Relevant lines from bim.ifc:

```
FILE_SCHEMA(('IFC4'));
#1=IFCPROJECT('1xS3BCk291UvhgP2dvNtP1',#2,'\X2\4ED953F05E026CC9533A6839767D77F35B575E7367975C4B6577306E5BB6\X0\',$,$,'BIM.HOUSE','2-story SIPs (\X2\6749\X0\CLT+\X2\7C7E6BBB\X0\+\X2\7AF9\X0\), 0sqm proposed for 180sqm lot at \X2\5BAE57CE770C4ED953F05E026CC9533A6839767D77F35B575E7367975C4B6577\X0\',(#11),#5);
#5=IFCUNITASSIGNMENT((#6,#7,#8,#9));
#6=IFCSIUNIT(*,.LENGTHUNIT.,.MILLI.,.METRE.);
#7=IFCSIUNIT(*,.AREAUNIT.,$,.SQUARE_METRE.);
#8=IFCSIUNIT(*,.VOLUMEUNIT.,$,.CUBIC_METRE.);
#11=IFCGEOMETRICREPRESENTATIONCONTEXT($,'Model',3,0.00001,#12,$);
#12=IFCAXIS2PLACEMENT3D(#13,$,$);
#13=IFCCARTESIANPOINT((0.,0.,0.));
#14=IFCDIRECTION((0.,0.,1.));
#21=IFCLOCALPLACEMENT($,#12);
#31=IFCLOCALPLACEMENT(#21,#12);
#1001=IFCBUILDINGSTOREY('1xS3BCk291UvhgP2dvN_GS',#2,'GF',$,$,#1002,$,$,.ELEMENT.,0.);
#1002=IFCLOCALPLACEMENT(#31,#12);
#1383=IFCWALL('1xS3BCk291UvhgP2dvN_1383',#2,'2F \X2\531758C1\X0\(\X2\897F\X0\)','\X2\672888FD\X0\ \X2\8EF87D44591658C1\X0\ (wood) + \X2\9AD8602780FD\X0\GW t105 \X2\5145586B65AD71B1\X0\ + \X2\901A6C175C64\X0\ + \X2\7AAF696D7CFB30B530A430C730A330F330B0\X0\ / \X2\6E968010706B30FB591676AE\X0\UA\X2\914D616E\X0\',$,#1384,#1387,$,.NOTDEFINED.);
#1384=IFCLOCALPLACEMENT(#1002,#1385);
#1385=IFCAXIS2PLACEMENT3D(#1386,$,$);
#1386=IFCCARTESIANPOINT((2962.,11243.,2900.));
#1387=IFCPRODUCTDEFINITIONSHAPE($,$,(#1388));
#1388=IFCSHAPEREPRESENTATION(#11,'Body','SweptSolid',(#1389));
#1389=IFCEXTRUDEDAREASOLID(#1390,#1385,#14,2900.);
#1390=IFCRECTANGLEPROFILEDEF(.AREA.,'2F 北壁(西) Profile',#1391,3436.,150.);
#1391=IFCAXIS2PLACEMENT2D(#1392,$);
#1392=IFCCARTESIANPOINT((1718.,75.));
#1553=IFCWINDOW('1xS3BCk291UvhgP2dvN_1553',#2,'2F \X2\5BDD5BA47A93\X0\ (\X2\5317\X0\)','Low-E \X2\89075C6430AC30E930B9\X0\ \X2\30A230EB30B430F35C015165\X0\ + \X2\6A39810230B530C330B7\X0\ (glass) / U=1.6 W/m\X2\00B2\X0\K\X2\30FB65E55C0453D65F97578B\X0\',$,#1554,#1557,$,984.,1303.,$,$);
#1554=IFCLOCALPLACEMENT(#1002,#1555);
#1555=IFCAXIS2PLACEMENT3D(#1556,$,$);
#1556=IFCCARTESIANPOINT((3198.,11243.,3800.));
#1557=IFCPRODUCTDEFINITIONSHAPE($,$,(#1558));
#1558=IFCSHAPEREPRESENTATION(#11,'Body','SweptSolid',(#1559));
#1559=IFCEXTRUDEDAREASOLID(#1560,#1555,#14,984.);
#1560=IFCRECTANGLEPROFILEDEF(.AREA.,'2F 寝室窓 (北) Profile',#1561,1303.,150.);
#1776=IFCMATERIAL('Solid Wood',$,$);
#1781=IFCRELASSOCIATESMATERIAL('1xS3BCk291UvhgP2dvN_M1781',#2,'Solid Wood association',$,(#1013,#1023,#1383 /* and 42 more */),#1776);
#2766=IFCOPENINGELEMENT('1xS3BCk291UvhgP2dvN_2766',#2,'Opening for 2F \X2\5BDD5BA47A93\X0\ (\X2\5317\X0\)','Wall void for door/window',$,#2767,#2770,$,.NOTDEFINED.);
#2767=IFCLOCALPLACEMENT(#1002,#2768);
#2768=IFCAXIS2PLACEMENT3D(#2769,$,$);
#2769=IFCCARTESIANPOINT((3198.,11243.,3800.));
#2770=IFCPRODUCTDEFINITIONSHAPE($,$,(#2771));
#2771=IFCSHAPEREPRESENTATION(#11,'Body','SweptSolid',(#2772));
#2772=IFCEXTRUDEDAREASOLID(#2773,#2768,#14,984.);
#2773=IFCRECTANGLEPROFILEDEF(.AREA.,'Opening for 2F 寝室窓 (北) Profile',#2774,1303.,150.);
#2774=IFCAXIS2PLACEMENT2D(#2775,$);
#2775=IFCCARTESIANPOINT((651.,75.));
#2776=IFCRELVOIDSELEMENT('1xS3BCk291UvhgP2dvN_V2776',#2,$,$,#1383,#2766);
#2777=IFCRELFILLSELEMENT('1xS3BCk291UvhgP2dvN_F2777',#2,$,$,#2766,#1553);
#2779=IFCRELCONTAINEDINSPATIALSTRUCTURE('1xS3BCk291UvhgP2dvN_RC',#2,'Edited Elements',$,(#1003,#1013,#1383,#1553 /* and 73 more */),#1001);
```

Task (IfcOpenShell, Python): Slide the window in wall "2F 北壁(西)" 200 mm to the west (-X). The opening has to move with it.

```python
import ifcopenshell
import ifcopenshell.api.geometry
import ifcopenshell.util.placement
import ifcopenshell.util.unit

model = ifcopenshell.open("bim.ifc")
unit_scale = ifcopenshell.util.unit.calculate_unit_scale(model)

window = model.by_id(1553)
opening = window.FillsVoids[0].RelatingOpeningElement
wall = opening.VoidsElements[0].RelatingBuildingElement

wall_matrix = ifcopenshell.util.placement.get_local_placement(wall.ObjectPlacement)
shift = wall_matrix[:3, 0] * -0.2 / unit_scale
before = ifcopenshell.util.placement.get_local_placement(window.ObjectPlacement)[:3, 3].copy()

# The window is not placed relative to its opening, so move both.
for product in (opening, window):
    matrix = ifcopenshell.util.placement.get_local_placement(product.ObjectPlacement)
    matrix[:3, 3] += shift
    ifcopenshell.api.geometry.edit_object_placement(model, product=product, matrix=matrix, is_si=False)

after = ifcopenshell.util.placement.get_local_placement(window.ObjectPlacement)[:3, 3]
print("window moved by", (after - before).round(3) + 0.0)

model.write("bim-out.ifc")
```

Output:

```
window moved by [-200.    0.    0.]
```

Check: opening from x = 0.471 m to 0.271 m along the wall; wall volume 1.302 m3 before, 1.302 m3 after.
